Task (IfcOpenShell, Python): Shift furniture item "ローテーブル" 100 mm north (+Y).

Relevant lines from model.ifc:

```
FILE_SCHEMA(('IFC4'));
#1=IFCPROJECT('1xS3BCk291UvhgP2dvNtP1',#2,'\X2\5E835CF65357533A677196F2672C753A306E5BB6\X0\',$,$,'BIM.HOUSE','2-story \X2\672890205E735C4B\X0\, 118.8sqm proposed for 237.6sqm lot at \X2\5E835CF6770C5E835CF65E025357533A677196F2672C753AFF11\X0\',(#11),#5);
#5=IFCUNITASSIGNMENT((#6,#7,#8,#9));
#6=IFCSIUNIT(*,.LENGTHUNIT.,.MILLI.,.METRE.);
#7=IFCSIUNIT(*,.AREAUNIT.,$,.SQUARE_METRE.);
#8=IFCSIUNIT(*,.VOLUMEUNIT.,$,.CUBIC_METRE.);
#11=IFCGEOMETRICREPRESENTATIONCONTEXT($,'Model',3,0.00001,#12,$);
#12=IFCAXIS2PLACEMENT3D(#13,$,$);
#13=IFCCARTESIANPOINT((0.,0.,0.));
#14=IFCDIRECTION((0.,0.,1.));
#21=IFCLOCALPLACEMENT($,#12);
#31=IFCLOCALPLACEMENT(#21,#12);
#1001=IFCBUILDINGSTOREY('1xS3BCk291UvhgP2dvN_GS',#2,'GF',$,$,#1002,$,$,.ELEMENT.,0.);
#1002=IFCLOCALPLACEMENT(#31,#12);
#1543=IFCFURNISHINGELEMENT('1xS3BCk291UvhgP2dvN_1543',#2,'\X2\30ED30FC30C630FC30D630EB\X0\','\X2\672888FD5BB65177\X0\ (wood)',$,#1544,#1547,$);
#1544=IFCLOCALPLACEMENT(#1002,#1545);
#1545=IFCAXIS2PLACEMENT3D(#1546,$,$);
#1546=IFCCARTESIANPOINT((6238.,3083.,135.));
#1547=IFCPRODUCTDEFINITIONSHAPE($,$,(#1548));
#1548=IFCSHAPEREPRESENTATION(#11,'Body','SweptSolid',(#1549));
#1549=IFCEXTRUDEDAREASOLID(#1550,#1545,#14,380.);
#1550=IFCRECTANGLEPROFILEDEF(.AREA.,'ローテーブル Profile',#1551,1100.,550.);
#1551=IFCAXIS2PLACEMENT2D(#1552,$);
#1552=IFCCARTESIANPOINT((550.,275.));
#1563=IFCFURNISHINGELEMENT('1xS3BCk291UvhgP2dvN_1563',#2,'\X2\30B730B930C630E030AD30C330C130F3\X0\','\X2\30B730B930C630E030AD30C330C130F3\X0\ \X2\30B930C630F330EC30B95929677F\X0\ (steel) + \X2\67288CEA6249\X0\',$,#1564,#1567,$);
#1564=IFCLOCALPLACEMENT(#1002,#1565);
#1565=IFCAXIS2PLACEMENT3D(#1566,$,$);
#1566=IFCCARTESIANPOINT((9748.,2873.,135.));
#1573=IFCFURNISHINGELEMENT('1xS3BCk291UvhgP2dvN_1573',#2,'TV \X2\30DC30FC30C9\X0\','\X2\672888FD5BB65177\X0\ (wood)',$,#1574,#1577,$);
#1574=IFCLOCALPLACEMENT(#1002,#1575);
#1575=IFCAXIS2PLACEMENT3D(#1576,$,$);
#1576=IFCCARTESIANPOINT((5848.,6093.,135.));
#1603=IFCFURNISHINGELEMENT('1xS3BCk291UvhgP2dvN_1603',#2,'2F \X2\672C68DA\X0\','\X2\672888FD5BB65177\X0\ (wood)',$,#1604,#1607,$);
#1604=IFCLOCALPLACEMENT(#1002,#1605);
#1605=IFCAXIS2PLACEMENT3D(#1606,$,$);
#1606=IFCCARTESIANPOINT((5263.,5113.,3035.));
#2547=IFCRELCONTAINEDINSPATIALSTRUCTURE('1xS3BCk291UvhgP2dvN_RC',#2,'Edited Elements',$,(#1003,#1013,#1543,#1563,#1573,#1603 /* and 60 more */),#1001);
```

```python
import ifcopenshell
import ifcopenshell.api.geometry
import ifcopenshell.util.placement

model = ifcopenshell.open("model.ifc")

item = model.by_guid("1xS3BCk291UvhgP2dvN_1543")
matrix = ifcopenshell.util.placement.get_local_placement(item.ObjectPlacement)
matrix[1, 3] += 100.0
ifcopenshell.api.geometry.edit_object_placement(model, product=item, matrix=matrix, is_si=False)

print(ifcopenshell.util.placement.get_local_placement(item.ObjectPlacement).round(3) + 0.0)

model.write("model_updated.ifc")
```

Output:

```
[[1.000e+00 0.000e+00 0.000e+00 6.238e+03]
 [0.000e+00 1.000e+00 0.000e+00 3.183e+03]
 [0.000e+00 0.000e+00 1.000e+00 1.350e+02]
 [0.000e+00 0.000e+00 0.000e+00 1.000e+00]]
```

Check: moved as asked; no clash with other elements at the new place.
